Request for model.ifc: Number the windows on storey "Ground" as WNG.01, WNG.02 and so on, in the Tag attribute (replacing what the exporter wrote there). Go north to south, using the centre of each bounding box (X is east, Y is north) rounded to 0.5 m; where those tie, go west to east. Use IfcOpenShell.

First a look at what the model holds.

```python
import ifcopenshell
import ifcopenshell.util.element
import ifcopenshell.util.placement

model = ifcopenshell.open("model.ifc")
print(model.schema)
storey = next(s for s in model.by_type("IfcBuildingStorey") if s.Name == "Ground")
windows = [e for e in ifcopenshell.util.element.get_decomposition(storey) if e.is_a("IfcWindow")]
for e in sorted(windows, key=lambda e: e.id()):
    origin = ifcopenshell.util.placement.get_local_placement(e.ObjectPlacement)[:3, 3]
    print(e.id(), e.Tag, e.Name, origin.round(2) + 0.0, sep=" | ")
```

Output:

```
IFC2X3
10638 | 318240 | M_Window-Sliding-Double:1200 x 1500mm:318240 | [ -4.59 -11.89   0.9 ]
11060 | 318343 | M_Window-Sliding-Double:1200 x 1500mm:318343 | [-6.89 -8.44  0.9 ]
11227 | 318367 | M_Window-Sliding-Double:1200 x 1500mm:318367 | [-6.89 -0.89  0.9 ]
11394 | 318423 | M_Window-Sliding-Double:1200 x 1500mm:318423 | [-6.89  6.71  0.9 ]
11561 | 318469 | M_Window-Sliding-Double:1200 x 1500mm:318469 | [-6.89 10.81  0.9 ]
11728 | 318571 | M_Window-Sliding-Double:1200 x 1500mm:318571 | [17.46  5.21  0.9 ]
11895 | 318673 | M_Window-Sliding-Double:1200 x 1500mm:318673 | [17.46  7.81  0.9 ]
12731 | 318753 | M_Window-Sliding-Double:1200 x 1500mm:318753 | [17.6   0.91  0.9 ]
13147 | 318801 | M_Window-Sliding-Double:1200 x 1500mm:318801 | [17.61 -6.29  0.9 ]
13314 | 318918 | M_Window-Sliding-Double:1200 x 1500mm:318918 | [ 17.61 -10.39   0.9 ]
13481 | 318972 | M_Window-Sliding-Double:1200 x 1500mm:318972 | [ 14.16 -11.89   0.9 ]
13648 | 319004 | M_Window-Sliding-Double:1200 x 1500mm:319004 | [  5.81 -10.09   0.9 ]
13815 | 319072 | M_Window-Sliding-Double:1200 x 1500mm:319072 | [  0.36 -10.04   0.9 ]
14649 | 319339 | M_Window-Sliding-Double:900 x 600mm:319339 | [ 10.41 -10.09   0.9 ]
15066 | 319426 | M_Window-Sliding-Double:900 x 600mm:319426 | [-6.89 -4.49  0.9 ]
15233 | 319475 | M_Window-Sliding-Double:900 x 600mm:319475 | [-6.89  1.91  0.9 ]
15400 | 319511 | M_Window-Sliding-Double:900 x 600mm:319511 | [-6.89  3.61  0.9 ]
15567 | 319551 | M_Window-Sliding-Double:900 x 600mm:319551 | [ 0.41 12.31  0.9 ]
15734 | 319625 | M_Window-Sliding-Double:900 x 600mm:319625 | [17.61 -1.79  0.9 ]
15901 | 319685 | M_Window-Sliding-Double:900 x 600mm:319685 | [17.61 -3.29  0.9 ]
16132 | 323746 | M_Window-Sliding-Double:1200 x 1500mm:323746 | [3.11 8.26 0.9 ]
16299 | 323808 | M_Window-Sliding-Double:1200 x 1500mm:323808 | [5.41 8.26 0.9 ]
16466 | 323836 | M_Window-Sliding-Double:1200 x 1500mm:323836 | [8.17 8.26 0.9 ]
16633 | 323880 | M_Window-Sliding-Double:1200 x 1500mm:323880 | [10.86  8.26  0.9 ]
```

```python
import ifcopenshell
import ifcopenshell.geom
import ifcopenshell.util.element
import ifcopenshell.util.shape

model = ifcopenshell.open("model.ifc")
settings = ifcopenshell.geom.settings()
settings.set("use-world-coords", True)


def centre(element):
    shape = ifcopenshell.geom.create_shape(settings, element)
    return ifcopenshell.util.shape.get_bbox_centroid(shape.geometry)


storey = next(s for s in model.by_type("IfcBuildingStorey") if s.Name == "Ground")
windows = [e for e in ifcopenshell.util.element.get_decomposition(storey) if e.is_a("IfcWindow")]

# Insertion points can sit at a corner or the storey origin, so sort by the geometry (in metres).
centres = {e: centre(e) for e in windows}
windows.sort(key=lambda e: (-round(centres[e][1] / 0.5), centres[e][0]))

for i, e in enumerate(windows, start=1):
    number = f"WNG.{i:02d}"
    e.Tag = number
    print(e.id(), number)

model.write("model_updated.ifc")
```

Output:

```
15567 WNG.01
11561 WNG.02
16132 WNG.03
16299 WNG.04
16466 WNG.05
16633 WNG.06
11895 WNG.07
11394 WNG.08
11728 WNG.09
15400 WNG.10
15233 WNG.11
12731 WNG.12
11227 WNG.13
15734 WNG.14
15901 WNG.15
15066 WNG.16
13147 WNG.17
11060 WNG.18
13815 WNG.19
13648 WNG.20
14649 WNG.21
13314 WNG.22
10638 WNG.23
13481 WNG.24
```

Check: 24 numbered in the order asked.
